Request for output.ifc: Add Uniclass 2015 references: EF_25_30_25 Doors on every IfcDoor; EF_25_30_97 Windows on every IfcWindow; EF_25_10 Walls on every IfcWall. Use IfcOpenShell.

First a look at what the model holds.

```python
import ifcopenshell

model = ifcopenshell.open("output.ifc")
print(model.schema)
print("classifications:", [c.Name for c in model.by_type("IfcClassification")])
for ifc_class in ("IfcDoor", "IfcRoof", "IfcStair", "IfcWall", "IfcWindow"):
    print(ifc_class, len(model.by_type(ifc_class)))
```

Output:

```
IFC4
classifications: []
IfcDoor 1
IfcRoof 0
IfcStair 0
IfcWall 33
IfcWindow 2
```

```python
import ifcopenshell
import ifcopenshell.api.classification

model = ifcopenshell.open("output.ifc")

system = ifcopenshell.api.classification.add_classification(model, classification="Uniclass 2015")

codes = {
    "IfcDoor": ("EF_25_30_25", "Doors"),
    "IfcWindow": ("EF_25_30_97", "Windows"),
    "IfcWall": ("EF_25_10", "Walls"),
}
for ifc_class, (code, name) in codes.items():
    products = model.by_type(ifc_class)
    ifcopenshell.api.classification.add_reference(
        model, products=products, classification=system, identification=code, name=name
    )
    print(code, len(products))

model.write("output_rev.ifc")
```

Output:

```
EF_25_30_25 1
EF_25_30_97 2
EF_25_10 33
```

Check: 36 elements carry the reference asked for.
